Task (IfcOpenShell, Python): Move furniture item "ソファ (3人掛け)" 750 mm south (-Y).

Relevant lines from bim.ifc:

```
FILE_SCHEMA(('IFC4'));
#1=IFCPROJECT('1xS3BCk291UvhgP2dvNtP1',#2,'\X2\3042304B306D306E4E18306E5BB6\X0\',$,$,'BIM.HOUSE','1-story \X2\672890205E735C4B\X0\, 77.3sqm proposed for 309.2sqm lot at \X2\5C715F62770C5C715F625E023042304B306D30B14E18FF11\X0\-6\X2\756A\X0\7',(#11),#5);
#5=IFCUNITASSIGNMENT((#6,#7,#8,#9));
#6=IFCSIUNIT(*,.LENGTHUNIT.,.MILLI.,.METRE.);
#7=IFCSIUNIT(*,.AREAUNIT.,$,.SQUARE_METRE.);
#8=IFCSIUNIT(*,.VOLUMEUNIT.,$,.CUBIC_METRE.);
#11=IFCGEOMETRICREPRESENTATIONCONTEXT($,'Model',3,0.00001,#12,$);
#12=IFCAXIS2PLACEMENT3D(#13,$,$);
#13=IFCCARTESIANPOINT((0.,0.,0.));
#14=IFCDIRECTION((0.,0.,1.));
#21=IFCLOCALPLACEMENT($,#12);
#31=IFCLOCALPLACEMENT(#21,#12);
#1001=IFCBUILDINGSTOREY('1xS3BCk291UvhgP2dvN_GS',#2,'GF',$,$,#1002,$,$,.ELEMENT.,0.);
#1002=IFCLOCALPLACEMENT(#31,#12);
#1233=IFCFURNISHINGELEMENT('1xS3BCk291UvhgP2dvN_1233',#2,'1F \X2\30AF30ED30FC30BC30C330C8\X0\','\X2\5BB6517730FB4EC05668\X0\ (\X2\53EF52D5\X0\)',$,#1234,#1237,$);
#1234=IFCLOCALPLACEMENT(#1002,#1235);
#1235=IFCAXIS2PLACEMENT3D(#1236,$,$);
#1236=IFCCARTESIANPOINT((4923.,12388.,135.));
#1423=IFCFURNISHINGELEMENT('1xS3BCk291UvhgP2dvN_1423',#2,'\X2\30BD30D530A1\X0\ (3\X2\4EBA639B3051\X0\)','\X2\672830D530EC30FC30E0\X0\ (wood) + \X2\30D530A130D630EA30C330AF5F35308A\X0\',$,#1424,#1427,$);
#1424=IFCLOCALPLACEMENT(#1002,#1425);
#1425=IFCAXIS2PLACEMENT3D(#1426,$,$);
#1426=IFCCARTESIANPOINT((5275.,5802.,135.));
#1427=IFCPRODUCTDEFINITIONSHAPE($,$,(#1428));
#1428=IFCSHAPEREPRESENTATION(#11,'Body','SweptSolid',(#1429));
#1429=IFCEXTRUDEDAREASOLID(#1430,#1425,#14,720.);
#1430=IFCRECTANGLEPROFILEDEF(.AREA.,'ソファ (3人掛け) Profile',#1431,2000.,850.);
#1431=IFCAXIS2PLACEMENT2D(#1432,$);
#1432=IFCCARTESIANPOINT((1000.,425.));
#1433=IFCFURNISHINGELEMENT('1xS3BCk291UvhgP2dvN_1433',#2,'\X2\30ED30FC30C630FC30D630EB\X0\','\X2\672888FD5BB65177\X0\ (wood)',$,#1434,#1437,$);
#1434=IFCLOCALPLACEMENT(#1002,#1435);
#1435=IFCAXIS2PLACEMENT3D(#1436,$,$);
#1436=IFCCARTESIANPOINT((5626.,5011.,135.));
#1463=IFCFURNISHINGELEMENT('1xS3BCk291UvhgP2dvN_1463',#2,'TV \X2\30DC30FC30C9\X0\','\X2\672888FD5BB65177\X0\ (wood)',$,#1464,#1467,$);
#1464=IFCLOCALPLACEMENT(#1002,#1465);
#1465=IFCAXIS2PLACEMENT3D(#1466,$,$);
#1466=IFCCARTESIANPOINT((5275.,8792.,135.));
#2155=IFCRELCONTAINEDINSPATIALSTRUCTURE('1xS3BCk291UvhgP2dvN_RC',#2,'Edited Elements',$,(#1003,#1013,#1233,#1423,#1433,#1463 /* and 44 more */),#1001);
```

```python
import ifcopenshell
import ifcopenshell.api.geometry
import ifcopenshell.util.placement
import ifcopenshell.util.unit

model = ifcopenshell.open("bim.ifc")
unit_scale = ifcopenshell.util.unit.calculate_unit_scale(model)

item = model.by_guid("1xS3BCk291UvhgP2dvN_1423")
matrix = ifcopenshell.util.placement.get_local_placement(item.ObjectPlacement)
matrix[1, 3] -= 0.75 / unit_scale
ifcopenshell.api.geometry.edit_object_placement(model, product=item, matrix=matrix, is_si=False)

print(ifcopenshell.util.placement.get_local_placement(item.ObjectPlacement).round(3) + 0.0)

model.write("bim_rev.ifc")
```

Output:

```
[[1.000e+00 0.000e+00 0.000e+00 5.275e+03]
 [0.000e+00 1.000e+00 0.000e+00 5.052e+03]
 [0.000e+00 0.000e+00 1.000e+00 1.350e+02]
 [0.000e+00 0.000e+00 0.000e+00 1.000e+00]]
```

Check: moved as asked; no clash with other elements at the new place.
